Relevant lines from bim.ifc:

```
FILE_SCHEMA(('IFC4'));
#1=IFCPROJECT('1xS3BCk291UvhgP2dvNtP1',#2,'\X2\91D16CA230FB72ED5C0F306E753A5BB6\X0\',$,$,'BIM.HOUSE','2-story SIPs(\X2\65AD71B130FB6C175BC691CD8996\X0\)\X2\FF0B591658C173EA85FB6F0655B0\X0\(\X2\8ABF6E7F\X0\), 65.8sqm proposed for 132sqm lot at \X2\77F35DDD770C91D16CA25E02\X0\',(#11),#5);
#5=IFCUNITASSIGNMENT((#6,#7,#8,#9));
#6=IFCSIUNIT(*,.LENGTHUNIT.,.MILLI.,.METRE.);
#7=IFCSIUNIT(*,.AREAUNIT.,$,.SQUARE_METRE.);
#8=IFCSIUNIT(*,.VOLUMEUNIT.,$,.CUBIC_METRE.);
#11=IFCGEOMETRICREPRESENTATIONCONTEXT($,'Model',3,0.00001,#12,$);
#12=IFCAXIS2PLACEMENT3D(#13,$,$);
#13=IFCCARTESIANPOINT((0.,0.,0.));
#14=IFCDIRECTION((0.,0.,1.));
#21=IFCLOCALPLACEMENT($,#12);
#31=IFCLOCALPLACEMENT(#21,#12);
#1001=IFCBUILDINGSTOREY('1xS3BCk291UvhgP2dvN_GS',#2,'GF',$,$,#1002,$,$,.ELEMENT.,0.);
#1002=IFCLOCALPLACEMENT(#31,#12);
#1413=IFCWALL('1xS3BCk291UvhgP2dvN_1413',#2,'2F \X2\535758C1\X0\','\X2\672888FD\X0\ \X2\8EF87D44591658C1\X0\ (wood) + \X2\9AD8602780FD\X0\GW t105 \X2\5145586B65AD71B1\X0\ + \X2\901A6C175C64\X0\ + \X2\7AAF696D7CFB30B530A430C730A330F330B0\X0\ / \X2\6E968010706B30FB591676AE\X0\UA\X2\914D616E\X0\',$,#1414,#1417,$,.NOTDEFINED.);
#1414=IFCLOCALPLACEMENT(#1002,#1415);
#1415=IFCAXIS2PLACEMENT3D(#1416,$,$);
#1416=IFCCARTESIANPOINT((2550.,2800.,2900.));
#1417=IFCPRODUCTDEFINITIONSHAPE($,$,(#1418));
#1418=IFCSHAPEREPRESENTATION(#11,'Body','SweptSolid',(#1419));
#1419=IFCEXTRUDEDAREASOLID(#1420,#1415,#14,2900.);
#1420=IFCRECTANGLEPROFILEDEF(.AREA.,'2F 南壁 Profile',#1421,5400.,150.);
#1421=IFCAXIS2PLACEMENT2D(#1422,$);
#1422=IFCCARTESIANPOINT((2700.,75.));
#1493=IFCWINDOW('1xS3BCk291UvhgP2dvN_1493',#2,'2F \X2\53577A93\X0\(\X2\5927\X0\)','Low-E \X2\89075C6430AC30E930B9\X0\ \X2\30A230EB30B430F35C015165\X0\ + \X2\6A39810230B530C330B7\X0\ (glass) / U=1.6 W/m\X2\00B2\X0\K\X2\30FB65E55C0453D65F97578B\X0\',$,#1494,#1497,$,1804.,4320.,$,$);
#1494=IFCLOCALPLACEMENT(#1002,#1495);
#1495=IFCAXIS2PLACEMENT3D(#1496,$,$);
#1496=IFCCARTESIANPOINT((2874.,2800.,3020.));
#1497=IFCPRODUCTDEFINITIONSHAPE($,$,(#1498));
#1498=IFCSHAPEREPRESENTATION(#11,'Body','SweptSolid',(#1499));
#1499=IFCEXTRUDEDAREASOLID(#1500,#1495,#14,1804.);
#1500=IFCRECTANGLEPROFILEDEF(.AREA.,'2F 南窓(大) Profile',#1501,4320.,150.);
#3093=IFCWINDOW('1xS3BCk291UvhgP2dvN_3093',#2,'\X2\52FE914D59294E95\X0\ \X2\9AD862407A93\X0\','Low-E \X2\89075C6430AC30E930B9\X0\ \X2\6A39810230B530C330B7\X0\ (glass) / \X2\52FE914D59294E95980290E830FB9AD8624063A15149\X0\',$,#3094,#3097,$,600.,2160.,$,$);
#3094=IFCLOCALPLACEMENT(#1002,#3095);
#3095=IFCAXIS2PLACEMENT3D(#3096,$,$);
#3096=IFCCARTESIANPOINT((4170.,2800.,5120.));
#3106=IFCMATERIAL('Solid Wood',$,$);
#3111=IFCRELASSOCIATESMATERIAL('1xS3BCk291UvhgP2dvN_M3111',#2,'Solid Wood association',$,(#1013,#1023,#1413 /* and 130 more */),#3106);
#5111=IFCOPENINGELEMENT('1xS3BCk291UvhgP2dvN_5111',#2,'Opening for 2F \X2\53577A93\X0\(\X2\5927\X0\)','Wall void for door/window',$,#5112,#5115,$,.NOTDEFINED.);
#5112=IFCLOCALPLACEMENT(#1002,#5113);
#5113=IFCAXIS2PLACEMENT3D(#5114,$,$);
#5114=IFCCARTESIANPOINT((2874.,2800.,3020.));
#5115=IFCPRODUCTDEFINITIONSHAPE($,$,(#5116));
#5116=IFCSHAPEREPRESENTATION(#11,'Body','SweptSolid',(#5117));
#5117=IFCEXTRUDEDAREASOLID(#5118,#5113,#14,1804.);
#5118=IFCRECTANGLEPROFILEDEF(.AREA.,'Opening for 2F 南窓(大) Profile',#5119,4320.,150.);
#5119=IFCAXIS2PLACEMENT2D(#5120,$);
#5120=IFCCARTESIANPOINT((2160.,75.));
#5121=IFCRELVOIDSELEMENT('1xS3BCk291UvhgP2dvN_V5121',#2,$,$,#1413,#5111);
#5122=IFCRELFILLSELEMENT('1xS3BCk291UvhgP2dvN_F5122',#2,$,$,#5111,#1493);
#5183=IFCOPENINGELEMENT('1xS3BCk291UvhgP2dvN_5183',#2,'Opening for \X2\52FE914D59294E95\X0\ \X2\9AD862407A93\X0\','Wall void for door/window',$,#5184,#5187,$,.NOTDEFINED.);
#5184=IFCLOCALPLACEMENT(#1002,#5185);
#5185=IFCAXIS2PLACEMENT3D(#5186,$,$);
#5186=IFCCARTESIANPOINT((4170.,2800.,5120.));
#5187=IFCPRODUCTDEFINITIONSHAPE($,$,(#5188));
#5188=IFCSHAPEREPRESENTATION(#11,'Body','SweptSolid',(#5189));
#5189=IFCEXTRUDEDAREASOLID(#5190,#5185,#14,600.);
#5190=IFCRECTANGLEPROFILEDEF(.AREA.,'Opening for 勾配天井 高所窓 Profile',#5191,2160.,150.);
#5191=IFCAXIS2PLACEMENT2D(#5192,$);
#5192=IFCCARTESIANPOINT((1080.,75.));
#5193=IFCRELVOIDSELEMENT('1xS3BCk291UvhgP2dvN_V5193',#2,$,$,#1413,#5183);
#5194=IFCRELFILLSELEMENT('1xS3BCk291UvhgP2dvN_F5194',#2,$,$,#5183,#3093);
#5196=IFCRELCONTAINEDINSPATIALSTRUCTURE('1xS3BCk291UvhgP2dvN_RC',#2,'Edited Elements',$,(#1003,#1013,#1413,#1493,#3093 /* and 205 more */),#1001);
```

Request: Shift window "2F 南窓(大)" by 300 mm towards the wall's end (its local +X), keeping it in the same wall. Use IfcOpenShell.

```python
import ifcopenshell
import ifcopenshell.api.geometry
import ifcopenshell.util.placement
import ifcopenshell.util.unit

model = ifcopenshell.open("bim.ifc")
unit_scale = ifcopenshell.util.unit.calculate_unit_scale(model)

window = model.by_id(1493)
opening = window.FillsVoids[0].RelatingOpeningElement
wall = opening.VoidsElements[0].RelatingBuildingElement

wall_matrix = ifcopenshell.util.placement.get_local_placement(wall.ObjectPlacement)
shift = wall_matrix[:3, 0] * 0.3 / unit_scale
before = ifcopenshell.util.placement.get_local_placement(window.ObjectPlacement)[:3, 3].copy()

# The window is not placed relative to its opening, so move both.
for product in (opening, window):
    matrix = ifcopenshell.util.placement.get_local_placement(product.ObjectPlacement)
    matrix[:3, 3] += shift
    ifcopenshell.api.geometry.edit_object_placement(model, product=product, matrix=matrix, is_si=False)

after = ifcopenshell.util.placement.get_local_placement(window.ObjectPlacement)[:3, 3]
print("window moved by", (after - before).round(3) + 0.0)

model.write("bim_rev.ifc")
```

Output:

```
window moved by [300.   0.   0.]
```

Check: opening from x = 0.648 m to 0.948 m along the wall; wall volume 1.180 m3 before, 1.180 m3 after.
